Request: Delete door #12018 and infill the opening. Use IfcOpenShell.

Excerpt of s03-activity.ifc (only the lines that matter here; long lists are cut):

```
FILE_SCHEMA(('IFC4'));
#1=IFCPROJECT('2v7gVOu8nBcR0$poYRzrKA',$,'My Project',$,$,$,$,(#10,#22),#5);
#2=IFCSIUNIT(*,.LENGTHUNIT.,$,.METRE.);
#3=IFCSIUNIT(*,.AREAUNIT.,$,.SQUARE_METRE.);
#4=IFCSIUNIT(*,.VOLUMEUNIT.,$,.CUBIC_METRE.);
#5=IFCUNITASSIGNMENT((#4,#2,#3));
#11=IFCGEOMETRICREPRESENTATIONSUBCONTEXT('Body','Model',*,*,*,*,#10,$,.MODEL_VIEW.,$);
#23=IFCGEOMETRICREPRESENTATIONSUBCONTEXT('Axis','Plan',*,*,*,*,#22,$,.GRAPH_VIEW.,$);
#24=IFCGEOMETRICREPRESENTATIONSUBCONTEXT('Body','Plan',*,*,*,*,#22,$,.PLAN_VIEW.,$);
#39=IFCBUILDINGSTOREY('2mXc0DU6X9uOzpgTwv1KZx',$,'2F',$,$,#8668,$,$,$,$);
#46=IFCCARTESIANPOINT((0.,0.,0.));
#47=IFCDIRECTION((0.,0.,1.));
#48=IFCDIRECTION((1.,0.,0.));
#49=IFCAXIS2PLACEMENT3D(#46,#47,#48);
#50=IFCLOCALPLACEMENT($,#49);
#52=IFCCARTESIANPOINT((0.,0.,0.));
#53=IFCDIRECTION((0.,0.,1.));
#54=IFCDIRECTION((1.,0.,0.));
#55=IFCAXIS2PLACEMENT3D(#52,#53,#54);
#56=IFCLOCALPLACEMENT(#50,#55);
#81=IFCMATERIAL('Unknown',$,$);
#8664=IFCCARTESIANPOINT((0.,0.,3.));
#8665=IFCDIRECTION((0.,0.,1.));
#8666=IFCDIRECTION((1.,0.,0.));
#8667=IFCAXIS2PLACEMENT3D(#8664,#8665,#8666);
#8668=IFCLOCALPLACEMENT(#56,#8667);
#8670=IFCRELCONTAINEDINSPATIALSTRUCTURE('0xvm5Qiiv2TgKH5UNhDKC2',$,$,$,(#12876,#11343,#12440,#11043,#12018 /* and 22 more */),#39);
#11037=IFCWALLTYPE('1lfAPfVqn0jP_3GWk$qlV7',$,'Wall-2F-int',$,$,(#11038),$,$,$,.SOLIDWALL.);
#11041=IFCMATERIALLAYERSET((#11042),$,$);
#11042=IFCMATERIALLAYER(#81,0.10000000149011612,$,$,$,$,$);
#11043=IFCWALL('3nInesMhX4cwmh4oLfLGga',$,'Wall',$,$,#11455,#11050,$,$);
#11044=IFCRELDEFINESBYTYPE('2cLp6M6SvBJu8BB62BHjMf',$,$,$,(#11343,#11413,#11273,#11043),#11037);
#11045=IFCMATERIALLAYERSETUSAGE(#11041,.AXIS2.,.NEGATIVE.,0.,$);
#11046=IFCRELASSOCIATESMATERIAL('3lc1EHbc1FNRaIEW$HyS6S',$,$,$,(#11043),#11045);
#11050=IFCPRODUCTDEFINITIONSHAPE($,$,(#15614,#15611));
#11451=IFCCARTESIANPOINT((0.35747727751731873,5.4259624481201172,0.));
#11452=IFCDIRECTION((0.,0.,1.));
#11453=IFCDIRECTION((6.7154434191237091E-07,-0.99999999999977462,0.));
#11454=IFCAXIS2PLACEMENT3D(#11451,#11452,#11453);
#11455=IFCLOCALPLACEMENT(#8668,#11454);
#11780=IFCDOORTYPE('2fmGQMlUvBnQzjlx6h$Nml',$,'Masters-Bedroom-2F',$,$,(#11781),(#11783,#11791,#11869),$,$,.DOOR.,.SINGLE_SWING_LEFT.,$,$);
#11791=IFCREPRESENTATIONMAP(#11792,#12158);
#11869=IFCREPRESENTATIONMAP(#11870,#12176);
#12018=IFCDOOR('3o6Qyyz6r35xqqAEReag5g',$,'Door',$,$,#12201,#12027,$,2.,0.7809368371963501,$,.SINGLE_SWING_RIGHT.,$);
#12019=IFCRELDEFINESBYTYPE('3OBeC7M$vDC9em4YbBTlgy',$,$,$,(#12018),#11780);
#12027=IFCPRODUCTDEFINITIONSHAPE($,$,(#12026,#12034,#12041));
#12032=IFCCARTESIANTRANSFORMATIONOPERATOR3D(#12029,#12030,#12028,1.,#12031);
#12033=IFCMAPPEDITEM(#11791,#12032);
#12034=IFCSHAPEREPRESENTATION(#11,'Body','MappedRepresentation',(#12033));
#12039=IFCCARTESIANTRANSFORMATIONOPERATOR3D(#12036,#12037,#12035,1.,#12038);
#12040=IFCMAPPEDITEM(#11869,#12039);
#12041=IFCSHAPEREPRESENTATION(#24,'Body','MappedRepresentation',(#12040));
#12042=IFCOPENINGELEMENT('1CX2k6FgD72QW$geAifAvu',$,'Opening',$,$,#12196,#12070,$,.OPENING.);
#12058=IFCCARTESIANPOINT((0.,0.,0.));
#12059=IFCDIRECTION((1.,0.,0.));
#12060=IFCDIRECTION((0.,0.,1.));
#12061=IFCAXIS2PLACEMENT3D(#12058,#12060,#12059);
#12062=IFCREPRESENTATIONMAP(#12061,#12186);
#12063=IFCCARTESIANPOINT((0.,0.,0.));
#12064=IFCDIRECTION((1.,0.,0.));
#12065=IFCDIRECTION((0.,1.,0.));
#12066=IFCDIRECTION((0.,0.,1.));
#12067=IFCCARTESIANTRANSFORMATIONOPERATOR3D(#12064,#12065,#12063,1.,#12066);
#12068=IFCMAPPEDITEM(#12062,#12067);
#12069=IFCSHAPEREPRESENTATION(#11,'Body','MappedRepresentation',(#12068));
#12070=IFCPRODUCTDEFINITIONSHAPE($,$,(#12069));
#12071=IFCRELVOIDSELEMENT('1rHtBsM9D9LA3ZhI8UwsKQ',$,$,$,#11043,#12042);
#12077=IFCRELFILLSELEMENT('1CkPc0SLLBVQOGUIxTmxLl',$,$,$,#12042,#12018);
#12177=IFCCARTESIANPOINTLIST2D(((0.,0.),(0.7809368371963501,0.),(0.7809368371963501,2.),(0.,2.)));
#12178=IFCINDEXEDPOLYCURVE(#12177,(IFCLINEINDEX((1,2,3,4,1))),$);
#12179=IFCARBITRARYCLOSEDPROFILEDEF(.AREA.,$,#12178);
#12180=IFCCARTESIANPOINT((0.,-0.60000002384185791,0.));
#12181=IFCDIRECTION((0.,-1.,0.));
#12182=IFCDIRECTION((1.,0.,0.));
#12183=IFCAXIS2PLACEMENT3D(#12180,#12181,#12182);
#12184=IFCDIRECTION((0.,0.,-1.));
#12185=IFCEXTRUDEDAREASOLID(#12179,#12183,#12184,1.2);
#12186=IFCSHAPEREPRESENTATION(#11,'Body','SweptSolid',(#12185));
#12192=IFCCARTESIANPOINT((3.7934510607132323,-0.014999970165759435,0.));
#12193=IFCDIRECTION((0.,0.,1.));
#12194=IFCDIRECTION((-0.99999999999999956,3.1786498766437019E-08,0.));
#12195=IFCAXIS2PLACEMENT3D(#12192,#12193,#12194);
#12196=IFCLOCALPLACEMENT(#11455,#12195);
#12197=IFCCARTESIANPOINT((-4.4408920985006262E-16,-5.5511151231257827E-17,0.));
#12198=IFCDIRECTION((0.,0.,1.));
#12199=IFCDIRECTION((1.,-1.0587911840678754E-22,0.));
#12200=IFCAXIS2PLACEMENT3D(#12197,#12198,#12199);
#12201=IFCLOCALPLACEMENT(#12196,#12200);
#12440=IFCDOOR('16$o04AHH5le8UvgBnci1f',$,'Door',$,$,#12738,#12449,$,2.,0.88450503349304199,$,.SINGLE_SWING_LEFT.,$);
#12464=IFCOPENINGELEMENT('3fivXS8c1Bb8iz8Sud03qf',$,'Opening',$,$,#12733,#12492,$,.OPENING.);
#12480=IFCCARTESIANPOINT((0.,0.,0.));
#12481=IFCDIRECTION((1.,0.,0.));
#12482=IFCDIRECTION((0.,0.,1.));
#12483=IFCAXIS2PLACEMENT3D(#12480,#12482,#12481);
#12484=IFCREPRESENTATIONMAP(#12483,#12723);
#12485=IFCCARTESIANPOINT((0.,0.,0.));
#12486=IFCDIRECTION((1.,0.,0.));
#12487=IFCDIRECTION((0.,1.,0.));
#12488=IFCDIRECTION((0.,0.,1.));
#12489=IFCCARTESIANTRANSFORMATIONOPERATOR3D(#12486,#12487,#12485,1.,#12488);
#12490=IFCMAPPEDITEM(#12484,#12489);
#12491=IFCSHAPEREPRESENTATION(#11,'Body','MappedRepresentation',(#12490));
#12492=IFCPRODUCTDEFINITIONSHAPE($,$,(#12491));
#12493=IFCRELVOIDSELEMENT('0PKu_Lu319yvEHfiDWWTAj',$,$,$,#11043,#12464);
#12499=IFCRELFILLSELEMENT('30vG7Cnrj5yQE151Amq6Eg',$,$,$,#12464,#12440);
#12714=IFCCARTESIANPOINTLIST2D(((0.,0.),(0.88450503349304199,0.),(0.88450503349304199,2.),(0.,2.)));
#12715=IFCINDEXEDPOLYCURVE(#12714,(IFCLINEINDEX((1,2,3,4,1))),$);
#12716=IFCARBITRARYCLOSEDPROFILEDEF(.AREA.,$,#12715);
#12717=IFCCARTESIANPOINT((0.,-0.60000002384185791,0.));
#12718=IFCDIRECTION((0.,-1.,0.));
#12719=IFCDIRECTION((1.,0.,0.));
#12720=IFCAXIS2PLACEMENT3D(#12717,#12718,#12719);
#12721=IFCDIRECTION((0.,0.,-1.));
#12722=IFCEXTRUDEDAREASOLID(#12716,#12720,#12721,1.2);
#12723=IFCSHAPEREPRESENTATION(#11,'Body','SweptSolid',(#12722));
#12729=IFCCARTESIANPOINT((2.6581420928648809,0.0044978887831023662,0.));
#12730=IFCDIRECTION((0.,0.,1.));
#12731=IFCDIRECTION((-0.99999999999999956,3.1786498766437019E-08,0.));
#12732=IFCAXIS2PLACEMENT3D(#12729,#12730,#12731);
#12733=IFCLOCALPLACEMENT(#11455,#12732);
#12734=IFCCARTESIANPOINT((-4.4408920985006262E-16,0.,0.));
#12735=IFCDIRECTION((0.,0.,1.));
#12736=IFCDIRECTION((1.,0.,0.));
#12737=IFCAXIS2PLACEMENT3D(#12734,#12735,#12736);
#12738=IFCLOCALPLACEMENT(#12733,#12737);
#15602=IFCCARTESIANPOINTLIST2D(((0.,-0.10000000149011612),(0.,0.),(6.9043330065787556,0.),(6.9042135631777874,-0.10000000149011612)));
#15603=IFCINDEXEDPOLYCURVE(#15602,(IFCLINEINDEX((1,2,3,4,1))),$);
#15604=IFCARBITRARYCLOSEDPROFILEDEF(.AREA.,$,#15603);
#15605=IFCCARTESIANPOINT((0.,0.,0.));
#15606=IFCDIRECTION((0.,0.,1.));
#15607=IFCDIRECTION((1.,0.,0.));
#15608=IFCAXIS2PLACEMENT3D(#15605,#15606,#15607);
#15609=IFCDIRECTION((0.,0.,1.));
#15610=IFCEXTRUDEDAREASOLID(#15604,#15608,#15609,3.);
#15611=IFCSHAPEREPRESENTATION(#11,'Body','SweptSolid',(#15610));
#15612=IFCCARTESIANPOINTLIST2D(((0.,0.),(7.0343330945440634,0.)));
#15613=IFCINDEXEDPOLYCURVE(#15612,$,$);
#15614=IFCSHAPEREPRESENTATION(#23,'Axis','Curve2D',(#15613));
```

```python
import ifcopenshell
import ifcopenshell.api.feature
import ifcopenshell.api.root
import ifcopenshell.geom
import ifcopenshell.util.shape

model = ifcopenshell.open("s03-activity.ifc")
settings = ifcopenshell.geom.settings()


def volume(element):
    """Net volume in cubic metres, openings subtracted."""
    shape = ifcopenshell.geom.create_shape(settings, element)
    return ifcopenshell.util.shape.get_volume(shape.geometry)


door = model.by_guid("3o6Qyyz6r35xqqAEReag5g")
opening = door.FillsVoids[0].RelatingOpeningElement
wall = opening.VoidsElements[0].RelatingBuildingElement
before = volume(wall)

ifcopenshell.api.root.remove_product(model, product=door)
ifcopenshell.api.feature.remove_feature(model, feature=opening)

after = volume(wall)

print(f"wall volume {before:.3f} -> {after:.3f} m3")

model.write("s03-activity_v2.ifc")
```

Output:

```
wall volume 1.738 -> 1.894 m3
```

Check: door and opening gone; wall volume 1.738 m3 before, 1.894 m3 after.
